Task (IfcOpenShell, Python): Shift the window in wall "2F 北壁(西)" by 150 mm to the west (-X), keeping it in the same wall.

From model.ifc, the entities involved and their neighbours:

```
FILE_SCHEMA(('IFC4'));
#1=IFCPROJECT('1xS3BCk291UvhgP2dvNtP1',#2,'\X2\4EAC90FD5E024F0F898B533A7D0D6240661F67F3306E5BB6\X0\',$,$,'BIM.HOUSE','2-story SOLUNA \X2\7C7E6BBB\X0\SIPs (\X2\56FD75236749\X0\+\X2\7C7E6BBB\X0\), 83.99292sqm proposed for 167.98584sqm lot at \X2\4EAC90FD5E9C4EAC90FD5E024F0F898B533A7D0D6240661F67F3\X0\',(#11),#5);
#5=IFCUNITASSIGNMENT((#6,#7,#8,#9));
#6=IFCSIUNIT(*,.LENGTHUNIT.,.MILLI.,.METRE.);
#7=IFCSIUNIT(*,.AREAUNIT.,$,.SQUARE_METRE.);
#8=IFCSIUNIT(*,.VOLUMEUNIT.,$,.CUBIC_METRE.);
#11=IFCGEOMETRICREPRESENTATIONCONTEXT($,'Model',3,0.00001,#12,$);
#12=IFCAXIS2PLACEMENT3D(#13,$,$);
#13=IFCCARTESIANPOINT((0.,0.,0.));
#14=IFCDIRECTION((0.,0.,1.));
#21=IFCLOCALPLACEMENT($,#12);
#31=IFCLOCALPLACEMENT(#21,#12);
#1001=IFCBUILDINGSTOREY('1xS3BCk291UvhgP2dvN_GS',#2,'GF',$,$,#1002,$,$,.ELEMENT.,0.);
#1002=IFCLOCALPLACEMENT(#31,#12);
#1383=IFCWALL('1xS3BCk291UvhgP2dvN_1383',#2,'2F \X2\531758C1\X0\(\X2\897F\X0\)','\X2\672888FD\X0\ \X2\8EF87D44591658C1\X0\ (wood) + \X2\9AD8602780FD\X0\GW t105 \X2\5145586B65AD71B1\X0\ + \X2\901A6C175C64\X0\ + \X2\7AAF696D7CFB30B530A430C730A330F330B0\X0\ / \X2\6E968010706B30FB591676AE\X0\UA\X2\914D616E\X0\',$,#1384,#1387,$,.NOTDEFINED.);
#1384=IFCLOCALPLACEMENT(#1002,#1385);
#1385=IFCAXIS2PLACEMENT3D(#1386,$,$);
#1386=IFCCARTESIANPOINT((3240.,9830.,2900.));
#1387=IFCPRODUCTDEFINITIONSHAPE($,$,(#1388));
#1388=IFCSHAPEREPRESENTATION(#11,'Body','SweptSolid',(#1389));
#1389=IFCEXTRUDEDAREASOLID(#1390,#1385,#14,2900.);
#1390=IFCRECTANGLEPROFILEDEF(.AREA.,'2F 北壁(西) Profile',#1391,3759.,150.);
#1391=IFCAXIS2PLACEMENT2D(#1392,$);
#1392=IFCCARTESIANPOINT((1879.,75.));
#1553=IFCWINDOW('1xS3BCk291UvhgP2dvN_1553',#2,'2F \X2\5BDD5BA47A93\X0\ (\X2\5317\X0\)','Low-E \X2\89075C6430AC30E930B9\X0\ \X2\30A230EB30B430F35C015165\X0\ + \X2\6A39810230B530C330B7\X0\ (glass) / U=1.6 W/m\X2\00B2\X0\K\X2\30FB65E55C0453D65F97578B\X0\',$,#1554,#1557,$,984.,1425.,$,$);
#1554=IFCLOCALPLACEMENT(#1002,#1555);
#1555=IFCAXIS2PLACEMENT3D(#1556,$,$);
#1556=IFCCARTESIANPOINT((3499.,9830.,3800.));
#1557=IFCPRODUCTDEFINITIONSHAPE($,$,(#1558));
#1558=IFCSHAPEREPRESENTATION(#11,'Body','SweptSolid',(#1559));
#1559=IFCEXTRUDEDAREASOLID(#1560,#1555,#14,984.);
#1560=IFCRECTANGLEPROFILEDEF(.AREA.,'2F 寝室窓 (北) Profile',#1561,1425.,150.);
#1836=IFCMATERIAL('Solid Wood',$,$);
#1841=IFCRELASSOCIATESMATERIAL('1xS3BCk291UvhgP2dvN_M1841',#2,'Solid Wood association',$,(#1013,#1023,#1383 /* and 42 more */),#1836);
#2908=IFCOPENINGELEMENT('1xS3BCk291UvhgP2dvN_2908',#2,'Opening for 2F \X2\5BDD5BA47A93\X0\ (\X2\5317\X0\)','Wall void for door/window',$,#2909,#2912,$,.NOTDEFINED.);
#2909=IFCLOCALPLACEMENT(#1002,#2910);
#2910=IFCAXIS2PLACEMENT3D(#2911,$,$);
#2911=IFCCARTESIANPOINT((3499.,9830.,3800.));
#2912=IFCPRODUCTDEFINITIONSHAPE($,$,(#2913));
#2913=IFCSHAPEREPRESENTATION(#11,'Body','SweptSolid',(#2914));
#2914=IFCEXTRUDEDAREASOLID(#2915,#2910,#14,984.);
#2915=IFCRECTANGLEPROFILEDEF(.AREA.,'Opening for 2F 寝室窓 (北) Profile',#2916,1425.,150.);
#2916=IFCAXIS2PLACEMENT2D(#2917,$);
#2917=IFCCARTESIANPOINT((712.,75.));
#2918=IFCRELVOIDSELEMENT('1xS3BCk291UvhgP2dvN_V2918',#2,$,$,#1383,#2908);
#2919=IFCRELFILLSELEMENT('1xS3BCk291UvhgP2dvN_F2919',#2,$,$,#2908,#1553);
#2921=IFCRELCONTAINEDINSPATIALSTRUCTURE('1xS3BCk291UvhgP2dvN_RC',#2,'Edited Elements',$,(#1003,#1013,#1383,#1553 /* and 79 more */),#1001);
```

```python
import ifcopenshell
import ifcopenshell.api.geometry
import ifcopenshell.util.placement
import ifcopenshell.util.unit

model = ifcopenshell.open("model.ifc")
unit_scale = ifcopenshell.util.unit.calculate_unit_scale(model)

window = model.by_guid("1xS3BCk291UvhgP2dvN_1553")
opening = window.FillsVoids[0].RelatingOpeningElement
wall = opening.VoidsElements[0].RelatingBuildingElement

wall_matrix = ifcopenshell.util.placement.get_local_placement(wall.ObjectPlacement)
shift = wall_matrix[:3, 0] * -0.15 / unit_scale
before = ifcopenshell.util.placement.get_local_placement(window.ObjectPlacement)[:3, 3].copy()

# The window is not placed relative to its opening, so move both.
for product in (opening, window):
    matrix = ifcopenshell.util.placement.get_local_placement(product.ObjectPlacement)
    matrix[:3, 3] += shift
    ifcopenshell.api.geometry.edit_object_placement(model, product=product, matrix=matrix, is_si=False)

after = ifcopenshell.util.placement.get_local_placement(window.ObjectPlacement)[:3, 3]
print("window moved by", (after - before).round(3) + 0.0)

model.write("model_v2.ifc")
```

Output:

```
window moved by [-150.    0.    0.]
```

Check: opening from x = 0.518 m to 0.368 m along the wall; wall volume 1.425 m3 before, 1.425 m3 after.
